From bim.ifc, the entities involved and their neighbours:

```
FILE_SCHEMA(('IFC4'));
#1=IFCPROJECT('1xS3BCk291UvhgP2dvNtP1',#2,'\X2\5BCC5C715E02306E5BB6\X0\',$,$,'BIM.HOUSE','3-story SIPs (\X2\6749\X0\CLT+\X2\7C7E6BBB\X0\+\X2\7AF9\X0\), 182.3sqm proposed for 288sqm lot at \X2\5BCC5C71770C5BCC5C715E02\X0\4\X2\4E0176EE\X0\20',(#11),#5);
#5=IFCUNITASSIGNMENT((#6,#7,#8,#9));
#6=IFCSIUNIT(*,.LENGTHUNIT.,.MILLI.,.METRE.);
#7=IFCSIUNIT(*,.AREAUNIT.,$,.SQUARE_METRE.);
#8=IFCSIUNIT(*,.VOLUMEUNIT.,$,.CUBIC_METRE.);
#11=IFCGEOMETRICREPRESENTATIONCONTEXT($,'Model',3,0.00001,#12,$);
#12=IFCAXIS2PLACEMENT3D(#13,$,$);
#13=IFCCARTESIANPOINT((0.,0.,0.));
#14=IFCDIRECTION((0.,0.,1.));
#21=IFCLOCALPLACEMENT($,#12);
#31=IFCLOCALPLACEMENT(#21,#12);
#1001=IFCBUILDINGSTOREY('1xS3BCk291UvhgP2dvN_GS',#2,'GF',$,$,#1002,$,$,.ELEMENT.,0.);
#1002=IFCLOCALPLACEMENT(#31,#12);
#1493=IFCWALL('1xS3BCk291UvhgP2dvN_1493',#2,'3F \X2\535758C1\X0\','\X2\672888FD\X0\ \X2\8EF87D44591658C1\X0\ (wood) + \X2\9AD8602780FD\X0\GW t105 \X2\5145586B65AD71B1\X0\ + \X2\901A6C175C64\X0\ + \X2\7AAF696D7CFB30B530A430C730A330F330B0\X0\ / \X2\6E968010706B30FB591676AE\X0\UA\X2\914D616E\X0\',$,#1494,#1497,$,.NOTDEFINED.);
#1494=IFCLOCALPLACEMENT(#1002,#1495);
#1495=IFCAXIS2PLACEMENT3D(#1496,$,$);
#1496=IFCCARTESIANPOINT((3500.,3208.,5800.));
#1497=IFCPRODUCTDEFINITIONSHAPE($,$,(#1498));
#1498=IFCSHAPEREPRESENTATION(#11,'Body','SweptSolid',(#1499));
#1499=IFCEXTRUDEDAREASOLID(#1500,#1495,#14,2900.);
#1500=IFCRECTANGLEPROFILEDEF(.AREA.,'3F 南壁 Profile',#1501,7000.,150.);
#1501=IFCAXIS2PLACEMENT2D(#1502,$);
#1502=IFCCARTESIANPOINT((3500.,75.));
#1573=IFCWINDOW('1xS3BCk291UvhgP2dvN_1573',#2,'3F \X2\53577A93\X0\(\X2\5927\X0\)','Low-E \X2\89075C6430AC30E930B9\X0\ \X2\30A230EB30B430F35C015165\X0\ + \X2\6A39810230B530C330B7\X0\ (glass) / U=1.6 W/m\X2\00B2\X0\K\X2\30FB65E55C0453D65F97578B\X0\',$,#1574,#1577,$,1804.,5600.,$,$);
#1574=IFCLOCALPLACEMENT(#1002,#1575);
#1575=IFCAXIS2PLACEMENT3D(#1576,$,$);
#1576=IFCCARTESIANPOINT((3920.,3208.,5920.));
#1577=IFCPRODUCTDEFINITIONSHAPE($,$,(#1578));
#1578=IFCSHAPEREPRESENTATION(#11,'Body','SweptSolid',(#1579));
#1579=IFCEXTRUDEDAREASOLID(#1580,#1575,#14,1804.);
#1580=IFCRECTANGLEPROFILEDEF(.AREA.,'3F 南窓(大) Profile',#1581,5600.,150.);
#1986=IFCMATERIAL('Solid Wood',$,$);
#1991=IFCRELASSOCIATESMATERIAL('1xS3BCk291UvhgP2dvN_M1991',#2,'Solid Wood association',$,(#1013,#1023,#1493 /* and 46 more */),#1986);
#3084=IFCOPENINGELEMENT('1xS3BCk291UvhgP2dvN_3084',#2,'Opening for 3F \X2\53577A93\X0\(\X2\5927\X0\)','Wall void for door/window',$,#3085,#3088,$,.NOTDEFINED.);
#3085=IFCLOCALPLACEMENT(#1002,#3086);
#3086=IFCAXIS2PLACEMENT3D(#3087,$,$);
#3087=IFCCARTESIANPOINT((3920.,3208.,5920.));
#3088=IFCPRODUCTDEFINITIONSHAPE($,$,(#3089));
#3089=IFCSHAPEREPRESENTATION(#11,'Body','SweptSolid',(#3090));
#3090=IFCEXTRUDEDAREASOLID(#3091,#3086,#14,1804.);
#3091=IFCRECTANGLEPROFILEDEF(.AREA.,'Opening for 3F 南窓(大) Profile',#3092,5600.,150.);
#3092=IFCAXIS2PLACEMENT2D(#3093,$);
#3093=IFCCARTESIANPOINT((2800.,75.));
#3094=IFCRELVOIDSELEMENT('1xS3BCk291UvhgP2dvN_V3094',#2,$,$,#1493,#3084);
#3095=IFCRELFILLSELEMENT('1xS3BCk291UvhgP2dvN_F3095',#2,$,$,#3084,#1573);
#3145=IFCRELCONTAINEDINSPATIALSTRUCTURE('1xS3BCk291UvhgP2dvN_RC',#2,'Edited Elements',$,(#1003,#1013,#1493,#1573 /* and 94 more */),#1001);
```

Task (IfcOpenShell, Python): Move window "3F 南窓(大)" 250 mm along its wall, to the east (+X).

```python
import ifcopenshell
import ifcopenshell.api.geometry
import ifcopenshell.util.placement
import ifcopenshell.util.unit

model = ifcopenshell.open("bim.ifc")
unit_scale = ifcopenshell.util.unit.calculate_unit_scale(model)

window = model.by_id(1573)
opening = window.FillsVoids[0].RelatingOpeningElement
wall = opening.VoidsElements[0].RelatingBuildingElement

wall_matrix = ifcopenshell.util.placement.get_local_placement(wall.ObjectPlacement)
shift = wall_matrix[:3, 0] * 0.25 / unit_scale
before = ifcopenshell.util.placement.get_local_placement(window.ObjectPlacement)[:3, 3].copy()

# The window is not placed relative to its opening, so move both.
for product in (opening, window):
    matrix = ifcopenshell.util.placement.get_local_placement(product.ObjectPlacement)
    matrix[:3, 3] += shift
    ifcopenshell.api.geometry.edit_object_placement(model, product=product, matrix=matrix, is_si=False)

after = ifcopenshell.util.placement.get_local_placement(window.ObjectPlacement)[:3, 3]
print("window moved by", (after - before).round(3) + 0.0)

model.write("bim_edited.ifc")
```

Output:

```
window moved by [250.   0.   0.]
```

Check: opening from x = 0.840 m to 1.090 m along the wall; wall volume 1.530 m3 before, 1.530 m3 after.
